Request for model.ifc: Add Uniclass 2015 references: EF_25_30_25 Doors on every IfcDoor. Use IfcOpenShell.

First a look at what the model holds.

```python
import ifcopenshell

model = ifcopenshell.open("model.ifc")
print(model.schema)
print("classifications:", [c.Name for c in model.by_type("IfcClassification")])
for ifc_class in ("IfcDoor", "IfcRoof", "IfcStair", "IfcWall", "IfcWindow"):
    print(ifc_class, len(model.by_type(ifc_class)))
```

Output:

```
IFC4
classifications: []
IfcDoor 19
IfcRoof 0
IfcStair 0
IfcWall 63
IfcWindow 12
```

```python
import ifcopenshell
import ifcopenshell.api.classification

model = ifcopenshell.open("model.ifc")

system = ifcopenshell.api.classification.add_classification(model, classification="Uniclass 2015")

codes = {
    "IfcDoor": ("EF_25_30_25", "Doors"),
}
for ifc_class, (code, name) in codes.items():
    products = model.by_type(ifc_class)
    ifcopenshell.api.classification.add_reference(
        model, products=products, classification=system, identification=code, name=name
    )
    print(code, len(products))

model.write("model-out.ifc")
```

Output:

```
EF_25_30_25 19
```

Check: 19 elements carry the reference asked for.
